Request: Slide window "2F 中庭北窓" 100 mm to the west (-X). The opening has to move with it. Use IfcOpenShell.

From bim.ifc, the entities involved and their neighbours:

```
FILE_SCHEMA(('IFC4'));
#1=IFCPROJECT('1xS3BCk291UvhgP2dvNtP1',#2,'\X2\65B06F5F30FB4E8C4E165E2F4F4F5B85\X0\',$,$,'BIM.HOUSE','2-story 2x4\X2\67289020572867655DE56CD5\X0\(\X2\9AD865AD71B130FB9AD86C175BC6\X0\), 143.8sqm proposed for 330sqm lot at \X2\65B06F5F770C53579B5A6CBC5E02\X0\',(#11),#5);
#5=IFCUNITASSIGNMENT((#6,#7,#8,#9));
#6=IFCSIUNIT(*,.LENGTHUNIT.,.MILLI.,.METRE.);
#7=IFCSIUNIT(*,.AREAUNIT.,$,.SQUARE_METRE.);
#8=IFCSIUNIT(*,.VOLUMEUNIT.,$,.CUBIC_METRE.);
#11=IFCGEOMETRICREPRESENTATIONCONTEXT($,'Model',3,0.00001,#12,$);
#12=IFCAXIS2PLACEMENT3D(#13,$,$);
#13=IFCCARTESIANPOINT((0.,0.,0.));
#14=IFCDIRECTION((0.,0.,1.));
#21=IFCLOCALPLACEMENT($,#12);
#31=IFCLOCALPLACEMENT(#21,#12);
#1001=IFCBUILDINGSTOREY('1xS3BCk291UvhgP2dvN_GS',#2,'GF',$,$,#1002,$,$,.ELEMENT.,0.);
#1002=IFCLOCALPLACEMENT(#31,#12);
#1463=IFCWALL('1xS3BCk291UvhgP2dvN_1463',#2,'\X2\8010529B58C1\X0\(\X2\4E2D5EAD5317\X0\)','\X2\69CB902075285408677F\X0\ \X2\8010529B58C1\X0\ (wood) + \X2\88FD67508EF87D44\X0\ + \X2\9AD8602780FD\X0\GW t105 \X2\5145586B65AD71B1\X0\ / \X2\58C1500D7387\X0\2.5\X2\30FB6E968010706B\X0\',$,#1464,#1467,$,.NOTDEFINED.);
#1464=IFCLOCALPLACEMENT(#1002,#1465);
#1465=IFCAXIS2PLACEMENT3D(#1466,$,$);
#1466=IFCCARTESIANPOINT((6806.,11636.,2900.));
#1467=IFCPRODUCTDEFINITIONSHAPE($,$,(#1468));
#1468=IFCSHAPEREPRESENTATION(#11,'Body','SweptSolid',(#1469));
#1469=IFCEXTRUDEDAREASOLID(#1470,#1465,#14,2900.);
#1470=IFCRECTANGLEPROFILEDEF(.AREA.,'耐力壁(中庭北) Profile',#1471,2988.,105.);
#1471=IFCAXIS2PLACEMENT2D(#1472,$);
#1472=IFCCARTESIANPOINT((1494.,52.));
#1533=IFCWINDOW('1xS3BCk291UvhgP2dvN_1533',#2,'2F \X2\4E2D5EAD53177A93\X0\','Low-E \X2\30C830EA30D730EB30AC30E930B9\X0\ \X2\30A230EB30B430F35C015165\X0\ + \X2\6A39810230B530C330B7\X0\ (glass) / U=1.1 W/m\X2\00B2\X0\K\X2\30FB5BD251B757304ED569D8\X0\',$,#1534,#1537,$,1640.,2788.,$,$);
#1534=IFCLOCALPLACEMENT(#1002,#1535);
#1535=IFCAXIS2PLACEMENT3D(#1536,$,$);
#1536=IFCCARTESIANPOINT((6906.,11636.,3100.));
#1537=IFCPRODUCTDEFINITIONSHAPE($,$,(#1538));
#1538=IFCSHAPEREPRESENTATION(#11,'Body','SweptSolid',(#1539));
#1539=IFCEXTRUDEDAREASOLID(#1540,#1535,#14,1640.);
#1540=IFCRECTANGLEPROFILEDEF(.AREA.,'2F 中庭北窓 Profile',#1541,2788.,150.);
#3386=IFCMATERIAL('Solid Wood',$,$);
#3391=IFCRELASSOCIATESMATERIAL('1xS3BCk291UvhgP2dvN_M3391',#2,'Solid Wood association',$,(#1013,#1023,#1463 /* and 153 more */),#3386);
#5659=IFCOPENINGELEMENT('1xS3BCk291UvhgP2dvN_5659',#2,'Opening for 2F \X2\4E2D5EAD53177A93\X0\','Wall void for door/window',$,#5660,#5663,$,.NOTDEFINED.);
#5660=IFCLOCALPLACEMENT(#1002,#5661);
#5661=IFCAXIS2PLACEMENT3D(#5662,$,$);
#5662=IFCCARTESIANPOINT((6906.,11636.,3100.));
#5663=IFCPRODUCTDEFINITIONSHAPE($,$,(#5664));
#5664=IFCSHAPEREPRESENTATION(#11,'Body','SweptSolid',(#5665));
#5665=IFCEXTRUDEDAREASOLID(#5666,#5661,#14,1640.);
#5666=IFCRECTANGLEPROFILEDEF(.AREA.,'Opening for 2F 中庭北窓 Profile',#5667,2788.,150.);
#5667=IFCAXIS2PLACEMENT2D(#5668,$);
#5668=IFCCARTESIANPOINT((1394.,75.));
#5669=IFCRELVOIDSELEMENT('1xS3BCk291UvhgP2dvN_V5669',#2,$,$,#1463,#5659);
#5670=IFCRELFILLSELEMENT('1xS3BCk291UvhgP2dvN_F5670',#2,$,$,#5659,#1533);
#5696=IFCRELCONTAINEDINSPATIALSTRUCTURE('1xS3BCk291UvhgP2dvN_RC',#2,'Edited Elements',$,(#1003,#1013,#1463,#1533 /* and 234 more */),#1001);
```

```python
import ifcopenshell
import ifcopenshell.api.geometry
import ifcopenshell.util.placement
import ifcopenshell.util.unit

model = ifcopenshell.open("bim.ifc")
unit_scale = ifcopenshell.util.unit.calculate_unit_scale(model)

window = model.by_guid("1xS3BCk291UvhgP2dvN_1533")
opening = window.FillsVoids[0].RelatingOpeningElement
wall = opening.VoidsElements[0].RelatingBuildingElement

wall_matrix = ifcopenshell.util.placement.get_local_placement(wall.ObjectPlacement)
shift = wall_matrix[:3, 0] * -0.1 / unit_scale
before = ifcopenshell.util.placement.get_local_placement(window.ObjectPlacement)[:3, 3].copy()

# The window is not placed relative to its opening, so move both.
for product in (opening, window):
    matrix = ifcopenshell.util.placement.get_local_placement(product.ObjectPlacement)
    matrix[:3, 3] += shift
    ifcopenshell.api.geometry.edit_object_placement(model, product=product, matrix=matrix, is_si=False)

after = ifcopenshell.util.placement.get_local_placement(window.ObjectPlacement)[:3, 3]
print("window moved by", (after - before).round(3) + 0.0)

model.write("bim_rev.ifc")
```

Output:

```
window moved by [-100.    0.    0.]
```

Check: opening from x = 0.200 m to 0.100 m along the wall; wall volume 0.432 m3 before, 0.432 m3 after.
